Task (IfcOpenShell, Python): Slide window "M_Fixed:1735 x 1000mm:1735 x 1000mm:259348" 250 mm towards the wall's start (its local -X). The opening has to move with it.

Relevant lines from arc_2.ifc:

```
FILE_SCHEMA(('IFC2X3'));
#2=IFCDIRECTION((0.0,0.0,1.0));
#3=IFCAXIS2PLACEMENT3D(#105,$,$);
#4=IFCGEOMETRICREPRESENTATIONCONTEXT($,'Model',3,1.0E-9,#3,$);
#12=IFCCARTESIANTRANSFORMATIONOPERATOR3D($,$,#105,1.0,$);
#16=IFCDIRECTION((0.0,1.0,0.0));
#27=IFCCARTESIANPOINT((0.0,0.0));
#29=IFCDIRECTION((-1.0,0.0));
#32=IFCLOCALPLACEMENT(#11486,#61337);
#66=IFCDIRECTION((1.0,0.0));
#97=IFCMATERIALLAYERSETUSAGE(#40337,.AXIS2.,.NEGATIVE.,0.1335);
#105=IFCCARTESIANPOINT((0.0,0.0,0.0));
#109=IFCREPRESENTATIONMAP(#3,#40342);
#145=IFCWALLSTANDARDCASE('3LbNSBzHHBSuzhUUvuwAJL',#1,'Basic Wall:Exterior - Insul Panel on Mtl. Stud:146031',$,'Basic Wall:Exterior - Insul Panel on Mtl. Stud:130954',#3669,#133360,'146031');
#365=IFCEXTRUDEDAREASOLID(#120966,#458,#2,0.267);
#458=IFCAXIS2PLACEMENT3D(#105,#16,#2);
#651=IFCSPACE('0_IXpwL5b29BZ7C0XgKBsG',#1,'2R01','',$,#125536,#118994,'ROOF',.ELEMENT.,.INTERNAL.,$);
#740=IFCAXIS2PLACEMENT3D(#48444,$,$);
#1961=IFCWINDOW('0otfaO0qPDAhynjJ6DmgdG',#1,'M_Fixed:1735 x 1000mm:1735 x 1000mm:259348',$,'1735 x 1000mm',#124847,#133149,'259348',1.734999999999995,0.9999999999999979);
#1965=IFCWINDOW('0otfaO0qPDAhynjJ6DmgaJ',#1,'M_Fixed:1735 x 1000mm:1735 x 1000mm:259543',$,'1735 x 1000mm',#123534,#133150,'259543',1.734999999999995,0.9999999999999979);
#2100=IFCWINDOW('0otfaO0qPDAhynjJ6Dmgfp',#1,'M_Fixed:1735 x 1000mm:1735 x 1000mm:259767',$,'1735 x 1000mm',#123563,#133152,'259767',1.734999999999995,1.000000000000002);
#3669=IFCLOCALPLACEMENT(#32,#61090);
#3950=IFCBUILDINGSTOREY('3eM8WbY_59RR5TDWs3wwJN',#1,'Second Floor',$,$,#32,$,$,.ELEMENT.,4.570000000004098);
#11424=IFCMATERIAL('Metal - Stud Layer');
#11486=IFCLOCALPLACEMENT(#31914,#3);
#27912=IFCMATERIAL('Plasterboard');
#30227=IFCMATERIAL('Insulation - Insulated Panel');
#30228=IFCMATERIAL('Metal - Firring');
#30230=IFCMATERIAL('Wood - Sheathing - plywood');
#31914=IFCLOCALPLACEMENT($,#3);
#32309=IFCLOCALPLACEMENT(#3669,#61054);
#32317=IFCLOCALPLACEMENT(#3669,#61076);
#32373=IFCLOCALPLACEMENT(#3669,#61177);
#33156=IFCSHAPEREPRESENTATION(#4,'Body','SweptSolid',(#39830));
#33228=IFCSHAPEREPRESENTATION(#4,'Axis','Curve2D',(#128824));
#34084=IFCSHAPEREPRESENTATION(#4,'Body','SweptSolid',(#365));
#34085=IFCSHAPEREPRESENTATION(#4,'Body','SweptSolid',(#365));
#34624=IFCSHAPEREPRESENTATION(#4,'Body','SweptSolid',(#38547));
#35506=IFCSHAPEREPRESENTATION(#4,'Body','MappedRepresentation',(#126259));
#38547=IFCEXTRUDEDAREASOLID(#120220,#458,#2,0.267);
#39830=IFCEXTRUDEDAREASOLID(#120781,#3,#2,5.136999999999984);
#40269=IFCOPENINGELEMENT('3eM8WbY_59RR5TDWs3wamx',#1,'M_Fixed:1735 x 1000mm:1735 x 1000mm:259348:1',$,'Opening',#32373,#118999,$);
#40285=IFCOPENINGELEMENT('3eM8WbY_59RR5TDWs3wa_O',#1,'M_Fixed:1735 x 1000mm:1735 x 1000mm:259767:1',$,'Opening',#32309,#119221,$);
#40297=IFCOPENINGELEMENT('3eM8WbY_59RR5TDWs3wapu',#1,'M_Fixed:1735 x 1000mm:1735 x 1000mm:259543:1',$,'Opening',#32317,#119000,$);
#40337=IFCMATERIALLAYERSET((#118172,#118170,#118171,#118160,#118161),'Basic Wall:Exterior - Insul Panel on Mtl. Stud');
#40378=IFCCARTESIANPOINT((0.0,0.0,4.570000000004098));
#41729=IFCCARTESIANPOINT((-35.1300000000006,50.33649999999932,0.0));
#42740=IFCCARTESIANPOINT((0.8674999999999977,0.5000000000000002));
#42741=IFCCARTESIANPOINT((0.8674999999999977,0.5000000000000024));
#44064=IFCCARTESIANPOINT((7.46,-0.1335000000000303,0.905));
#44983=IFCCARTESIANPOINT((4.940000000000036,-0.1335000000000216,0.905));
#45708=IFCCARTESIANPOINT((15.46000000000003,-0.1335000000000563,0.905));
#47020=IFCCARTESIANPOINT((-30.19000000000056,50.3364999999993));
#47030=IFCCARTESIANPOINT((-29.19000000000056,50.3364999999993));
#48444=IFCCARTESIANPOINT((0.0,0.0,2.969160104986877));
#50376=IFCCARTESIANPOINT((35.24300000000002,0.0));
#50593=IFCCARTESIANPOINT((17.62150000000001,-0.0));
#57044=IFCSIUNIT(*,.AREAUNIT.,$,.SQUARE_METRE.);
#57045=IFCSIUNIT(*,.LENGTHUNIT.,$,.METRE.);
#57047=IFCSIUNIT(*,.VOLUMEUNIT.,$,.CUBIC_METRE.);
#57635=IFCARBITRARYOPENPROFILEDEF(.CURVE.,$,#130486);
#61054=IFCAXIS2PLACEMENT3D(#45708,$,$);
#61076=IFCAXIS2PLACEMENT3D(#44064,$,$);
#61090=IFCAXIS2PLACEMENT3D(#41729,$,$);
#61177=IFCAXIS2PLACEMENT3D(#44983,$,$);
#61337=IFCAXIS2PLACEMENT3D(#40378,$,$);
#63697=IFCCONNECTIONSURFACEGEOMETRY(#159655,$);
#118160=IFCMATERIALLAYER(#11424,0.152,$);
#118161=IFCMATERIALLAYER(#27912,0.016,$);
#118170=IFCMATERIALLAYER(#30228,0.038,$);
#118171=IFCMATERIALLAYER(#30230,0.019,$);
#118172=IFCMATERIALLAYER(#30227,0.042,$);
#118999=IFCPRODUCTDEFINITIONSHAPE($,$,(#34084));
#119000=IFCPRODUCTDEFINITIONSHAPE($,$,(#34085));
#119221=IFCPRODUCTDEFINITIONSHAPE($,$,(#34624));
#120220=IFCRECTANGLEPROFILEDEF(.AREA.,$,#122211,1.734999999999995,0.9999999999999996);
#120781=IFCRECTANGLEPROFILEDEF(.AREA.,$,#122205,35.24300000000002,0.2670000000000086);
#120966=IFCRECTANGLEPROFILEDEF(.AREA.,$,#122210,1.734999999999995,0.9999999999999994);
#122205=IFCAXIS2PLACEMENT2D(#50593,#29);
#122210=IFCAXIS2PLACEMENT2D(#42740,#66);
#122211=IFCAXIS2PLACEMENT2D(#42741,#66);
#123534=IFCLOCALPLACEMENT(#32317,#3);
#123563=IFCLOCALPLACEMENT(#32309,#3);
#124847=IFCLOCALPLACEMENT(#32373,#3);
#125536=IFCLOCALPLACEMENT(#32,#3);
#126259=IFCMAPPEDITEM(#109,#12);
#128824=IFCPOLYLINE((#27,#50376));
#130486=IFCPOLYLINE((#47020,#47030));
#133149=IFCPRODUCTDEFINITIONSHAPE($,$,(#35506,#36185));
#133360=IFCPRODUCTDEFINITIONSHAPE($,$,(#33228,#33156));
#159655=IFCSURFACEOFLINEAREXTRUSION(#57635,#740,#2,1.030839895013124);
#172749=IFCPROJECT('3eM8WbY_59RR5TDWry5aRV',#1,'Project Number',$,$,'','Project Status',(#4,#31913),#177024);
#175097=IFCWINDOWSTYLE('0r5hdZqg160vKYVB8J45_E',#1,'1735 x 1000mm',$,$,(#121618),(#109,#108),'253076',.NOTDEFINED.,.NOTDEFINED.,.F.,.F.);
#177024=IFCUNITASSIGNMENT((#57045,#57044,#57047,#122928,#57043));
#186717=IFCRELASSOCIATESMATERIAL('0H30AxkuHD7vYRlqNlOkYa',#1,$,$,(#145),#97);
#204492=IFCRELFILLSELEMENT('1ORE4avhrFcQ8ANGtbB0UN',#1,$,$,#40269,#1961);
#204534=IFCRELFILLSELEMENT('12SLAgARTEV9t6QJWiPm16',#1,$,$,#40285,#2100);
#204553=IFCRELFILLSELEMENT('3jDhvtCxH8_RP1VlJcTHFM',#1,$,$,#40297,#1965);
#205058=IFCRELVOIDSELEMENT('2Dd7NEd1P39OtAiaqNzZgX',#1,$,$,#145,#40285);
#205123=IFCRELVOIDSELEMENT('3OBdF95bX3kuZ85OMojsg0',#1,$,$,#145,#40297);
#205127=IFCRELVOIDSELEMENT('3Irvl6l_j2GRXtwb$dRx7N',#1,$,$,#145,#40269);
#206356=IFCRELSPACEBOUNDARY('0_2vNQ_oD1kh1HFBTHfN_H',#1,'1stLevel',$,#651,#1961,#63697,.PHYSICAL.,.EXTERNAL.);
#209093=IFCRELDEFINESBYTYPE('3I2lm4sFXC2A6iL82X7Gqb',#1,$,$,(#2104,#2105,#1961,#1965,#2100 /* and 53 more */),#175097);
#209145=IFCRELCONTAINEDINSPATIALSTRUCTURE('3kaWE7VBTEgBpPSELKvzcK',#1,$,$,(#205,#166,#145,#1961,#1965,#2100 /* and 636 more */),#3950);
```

```python
import numpy as np
import ifcopenshell
import ifcopenshell.api.geometry
import ifcopenshell.util.placement

model = ifcopenshell.open("arc_2.ifc")

window = model.by_id(1961)
opening = window.FillsVoids[0].RelatingOpeningElement
wall = opening.VoidsElements[0].RelatingBuildingElement

wall_matrix = ifcopenshell.util.placement.get_local_placement(wall.ObjectPlacement)
shift = wall_matrix[:3, 0] * -0.25
before = ifcopenshell.util.placement.get_local_placement(window.ObjectPlacement)[:3, 3].copy()

# The window is placed relative to its opening, so it follows when the opening moves.
matrix = ifcopenshell.util.placement.get_local_placement(opening.ObjectPlacement)
matrix[:3, 3] += shift
ifcopenshell.api.geometry.edit_object_placement(
    model, product=opening, matrix=matrix, is_si=False, should_transform_children=True
)

# Space boundary surfaces are stored in each space's coordinates; move them too.
for rel in window.ProvidesBoundaries:
    if not rel.ConnectionGeometry:
        continue
    surface = rel.ConnectionGeometry.SurfaceOnRelatingElement
    space_matrix = ifcopenshell.util.placement.get_local_placement(rel.RelatingSpace.ObjectPlacement)
    point = np.array(surface.Position.Location.Coordinates) + space_matrix[:3, :3].T @ shift
    surface.Position = model.createIfcAxis2Placement3D(
        model.createIfcCartesianPoint(point.tolist()), surface.Position.Axis, surface.Position.RefDirection
    )

after = ifcopenshell.util.placement.get_local_placement(window.ObjectPlacement)[:3, 3]
print("window moved by", (after - before).round(3) + 0.0)

model.write("arc_2_v2.ifc")
```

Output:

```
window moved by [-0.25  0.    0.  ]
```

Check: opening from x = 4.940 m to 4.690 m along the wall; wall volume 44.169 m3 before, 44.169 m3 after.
